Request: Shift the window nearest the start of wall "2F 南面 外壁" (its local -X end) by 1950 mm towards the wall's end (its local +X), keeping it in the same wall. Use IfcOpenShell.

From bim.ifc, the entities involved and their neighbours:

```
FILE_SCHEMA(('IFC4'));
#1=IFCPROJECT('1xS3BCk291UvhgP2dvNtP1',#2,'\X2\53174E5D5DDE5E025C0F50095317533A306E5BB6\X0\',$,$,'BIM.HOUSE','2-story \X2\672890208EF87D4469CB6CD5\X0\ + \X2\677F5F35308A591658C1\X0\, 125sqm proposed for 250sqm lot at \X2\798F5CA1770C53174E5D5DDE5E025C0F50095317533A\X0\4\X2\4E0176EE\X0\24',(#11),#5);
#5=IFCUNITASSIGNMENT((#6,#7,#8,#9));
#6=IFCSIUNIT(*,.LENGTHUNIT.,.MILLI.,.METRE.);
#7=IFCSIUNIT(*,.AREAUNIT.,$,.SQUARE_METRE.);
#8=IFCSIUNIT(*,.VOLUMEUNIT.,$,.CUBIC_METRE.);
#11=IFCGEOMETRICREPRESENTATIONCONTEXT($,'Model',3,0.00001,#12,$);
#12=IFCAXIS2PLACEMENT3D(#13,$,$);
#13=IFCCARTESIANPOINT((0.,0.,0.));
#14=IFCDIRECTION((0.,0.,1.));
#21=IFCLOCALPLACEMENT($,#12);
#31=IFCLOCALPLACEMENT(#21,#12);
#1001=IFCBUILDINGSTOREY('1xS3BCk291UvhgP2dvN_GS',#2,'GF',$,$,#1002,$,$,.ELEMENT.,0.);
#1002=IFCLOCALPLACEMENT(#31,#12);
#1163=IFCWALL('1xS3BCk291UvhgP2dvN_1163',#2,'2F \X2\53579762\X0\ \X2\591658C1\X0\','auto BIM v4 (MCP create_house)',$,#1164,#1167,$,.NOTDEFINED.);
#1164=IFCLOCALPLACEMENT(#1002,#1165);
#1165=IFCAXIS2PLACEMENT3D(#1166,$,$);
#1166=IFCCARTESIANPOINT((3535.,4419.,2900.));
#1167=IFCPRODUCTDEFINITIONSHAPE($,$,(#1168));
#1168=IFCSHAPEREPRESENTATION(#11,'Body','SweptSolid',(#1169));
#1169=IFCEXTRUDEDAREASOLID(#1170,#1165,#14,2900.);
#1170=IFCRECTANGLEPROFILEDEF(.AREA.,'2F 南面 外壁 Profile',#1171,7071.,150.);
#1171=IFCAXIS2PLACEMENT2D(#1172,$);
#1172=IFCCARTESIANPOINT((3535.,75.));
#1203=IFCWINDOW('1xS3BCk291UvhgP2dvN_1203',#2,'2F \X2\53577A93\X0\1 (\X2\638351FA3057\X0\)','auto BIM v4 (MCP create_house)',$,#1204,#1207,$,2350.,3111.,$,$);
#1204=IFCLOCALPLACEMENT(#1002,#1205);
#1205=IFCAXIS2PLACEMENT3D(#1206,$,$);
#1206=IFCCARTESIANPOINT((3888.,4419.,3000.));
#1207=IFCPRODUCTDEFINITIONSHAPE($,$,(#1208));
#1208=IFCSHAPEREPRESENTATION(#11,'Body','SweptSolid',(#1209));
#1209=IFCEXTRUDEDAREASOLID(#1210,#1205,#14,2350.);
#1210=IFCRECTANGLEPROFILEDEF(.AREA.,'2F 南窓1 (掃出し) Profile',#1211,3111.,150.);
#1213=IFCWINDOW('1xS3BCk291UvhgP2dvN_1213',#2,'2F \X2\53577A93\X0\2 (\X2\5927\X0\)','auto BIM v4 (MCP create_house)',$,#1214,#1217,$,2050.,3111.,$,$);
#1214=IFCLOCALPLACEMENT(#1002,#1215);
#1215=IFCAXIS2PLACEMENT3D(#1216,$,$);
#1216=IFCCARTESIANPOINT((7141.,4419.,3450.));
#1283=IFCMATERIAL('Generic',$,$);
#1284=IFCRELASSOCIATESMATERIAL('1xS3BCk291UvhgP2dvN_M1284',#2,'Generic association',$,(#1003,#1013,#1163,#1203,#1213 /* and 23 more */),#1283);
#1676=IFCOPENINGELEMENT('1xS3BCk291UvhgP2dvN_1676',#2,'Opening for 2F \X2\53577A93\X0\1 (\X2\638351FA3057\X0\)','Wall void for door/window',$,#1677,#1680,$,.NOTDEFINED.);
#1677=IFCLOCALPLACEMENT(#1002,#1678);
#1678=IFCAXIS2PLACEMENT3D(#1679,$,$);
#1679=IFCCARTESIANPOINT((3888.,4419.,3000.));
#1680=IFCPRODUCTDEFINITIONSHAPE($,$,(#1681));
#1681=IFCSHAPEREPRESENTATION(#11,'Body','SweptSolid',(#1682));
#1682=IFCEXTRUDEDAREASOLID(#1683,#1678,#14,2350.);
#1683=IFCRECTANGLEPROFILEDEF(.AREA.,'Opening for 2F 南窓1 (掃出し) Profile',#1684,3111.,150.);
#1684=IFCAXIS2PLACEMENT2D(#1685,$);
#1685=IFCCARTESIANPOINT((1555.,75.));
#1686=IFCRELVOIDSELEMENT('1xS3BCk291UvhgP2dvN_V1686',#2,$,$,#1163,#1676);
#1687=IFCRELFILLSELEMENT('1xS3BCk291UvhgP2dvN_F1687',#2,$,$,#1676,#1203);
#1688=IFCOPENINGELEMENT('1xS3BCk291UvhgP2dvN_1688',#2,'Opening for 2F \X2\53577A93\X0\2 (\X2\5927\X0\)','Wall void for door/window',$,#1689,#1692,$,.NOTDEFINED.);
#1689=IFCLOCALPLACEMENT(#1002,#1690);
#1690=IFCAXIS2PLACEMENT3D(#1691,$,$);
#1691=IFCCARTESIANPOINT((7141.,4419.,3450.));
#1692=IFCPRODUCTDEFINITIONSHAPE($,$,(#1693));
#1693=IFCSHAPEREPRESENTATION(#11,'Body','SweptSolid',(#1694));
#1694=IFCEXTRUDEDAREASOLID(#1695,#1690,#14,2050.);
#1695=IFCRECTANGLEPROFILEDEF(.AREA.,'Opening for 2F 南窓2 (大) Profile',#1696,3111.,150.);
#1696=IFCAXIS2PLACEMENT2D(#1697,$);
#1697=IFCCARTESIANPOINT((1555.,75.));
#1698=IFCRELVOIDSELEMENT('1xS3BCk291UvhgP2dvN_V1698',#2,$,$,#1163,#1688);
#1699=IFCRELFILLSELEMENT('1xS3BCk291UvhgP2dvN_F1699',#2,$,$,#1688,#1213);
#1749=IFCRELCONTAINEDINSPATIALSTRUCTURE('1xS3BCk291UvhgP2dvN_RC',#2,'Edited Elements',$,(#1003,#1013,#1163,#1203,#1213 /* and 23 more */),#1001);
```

```python
import ifcopenshell
import ifcopenshell.api.geometry
import ifcopenshell.util.placement
import ifcopenshell.util.unit

model = ifcopenshell.open("bim.ifc")
unit_scale = ifcopenshell.util.unit.calculate_unit_scale(model)

window = model.by_guid("1xS3BCk291UvhgP2dvN_1203")
opening = window.FillsVoids[0].RelatingOpeningElement
wall = opening.VoidsElements[0].RelatingBuildingElement

wall_matrix = ifcopenshell.util.placement.get_local_placement(wall.ObjectPlacement)
shift = wall_matrix[:3, 0] * 1.95 / unit_scale
before = ifcopenshell.util.placement.get_local_placement(window.ObjectPlacement)[:3, 3].copy()

# The window is not placed relative to its opening, so move both.
for product in (opening, window):
    matrix = ifcopenshell.util.placement.get_local_placement(product.ObjectPlacement)
    matrix[:3, 3] += shift
    ifcopenshell.api.geometry.edit_object_placement(model, product=product, matrix=matrix, is_si=False)

after = ifcopenshell.util.placement.get_local_placement(window.ObjectPlacement)[:3, 3]
print("window moved by", (after - before).round(3) + 0.0)

model.write("bim_rev.ifc")
```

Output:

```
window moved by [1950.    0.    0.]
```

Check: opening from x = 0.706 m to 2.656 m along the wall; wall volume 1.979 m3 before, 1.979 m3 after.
